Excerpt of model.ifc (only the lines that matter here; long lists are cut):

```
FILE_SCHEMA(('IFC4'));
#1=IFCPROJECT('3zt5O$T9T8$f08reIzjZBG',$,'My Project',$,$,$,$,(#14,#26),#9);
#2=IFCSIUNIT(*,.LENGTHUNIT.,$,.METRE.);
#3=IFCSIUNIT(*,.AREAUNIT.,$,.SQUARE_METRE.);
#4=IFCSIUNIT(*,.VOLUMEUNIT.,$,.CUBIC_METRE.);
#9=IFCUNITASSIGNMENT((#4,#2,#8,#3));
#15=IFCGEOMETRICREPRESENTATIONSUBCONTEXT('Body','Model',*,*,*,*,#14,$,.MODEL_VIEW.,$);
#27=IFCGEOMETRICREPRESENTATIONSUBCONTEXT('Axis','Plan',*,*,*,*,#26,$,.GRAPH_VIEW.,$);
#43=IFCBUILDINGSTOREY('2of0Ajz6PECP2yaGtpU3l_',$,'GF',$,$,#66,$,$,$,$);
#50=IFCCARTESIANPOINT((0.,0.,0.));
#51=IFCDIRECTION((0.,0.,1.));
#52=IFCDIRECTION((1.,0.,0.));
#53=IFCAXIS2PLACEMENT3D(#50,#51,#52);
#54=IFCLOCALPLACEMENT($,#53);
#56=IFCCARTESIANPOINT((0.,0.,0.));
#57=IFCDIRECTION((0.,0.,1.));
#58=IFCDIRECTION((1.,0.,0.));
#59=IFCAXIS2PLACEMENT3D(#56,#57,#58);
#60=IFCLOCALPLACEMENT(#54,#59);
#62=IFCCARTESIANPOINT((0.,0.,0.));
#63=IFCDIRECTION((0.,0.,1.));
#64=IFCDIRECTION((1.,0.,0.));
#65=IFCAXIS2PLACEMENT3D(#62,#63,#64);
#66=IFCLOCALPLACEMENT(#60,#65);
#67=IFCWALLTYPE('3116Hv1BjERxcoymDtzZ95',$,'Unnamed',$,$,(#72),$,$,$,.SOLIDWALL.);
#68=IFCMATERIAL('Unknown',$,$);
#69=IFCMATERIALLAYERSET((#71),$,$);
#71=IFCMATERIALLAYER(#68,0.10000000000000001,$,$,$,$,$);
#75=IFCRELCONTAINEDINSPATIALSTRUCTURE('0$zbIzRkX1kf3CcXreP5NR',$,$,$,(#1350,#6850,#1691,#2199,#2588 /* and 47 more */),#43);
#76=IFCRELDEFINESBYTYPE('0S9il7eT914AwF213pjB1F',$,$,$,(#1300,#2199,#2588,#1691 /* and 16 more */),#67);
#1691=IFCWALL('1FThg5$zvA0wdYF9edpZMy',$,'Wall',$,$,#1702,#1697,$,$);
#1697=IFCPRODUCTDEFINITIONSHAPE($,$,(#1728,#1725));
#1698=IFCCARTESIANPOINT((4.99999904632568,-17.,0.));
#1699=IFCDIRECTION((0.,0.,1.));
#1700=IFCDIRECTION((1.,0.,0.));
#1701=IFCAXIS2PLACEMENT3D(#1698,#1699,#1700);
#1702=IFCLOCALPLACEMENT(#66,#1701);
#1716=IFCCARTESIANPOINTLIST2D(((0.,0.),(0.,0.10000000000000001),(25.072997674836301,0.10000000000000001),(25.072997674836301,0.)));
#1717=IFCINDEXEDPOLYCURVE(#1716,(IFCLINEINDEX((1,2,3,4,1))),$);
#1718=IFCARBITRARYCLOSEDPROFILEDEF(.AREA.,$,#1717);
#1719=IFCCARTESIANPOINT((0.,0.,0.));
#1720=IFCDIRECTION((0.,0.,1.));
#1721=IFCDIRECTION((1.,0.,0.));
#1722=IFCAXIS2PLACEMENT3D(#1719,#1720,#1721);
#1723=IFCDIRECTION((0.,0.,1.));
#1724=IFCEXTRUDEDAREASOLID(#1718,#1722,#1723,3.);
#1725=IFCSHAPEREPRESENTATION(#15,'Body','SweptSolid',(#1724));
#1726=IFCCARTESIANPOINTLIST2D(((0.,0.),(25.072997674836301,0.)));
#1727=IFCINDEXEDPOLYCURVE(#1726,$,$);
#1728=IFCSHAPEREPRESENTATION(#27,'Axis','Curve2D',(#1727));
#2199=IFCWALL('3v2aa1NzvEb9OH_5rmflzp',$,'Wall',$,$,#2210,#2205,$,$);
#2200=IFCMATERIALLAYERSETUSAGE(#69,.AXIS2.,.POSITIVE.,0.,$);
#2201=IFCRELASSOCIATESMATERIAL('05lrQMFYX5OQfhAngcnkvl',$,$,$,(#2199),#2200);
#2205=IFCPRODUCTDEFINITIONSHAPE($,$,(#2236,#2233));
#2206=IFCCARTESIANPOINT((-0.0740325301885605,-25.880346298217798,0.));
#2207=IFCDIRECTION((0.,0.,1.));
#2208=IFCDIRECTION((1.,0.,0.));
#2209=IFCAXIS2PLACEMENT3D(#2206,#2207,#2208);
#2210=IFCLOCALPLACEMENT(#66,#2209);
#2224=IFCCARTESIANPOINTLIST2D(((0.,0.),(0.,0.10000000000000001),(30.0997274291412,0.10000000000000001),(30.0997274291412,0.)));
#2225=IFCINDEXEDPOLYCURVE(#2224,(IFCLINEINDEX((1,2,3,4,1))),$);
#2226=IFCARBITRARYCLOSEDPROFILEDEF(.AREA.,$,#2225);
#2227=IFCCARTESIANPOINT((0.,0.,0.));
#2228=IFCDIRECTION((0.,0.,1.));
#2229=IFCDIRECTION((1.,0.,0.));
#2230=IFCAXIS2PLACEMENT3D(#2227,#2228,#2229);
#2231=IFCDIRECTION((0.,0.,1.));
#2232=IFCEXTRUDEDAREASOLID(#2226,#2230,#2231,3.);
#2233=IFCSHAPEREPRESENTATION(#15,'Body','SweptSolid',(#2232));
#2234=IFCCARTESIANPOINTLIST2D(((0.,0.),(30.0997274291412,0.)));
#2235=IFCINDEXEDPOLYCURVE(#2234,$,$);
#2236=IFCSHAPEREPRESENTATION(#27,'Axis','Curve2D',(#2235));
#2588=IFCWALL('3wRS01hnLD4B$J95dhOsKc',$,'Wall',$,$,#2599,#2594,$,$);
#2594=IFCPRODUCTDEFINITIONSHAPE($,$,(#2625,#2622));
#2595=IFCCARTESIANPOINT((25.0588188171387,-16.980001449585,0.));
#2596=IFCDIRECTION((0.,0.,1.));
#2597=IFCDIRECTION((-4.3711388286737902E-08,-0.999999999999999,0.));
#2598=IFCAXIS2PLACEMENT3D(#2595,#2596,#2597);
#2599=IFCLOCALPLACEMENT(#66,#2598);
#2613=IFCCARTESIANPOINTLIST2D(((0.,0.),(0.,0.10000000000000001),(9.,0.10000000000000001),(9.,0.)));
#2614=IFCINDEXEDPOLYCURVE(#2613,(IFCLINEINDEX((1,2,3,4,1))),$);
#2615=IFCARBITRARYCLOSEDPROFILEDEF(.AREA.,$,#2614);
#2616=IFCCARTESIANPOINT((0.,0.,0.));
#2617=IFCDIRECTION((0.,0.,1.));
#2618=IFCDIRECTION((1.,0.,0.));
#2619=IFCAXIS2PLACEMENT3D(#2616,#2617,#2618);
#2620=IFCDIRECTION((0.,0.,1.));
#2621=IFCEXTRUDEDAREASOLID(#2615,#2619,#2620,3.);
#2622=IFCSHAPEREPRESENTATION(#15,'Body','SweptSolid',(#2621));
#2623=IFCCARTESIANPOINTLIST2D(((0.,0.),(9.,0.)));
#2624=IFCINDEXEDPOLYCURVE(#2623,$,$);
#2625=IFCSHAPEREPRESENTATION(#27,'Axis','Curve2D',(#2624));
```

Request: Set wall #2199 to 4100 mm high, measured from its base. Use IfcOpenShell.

```python
import ifcopenshell
import ifcopenshell.geom
import ifcopenshell.util.representation
import ifcopenshell.util.shape

model = ifcopenshell.open("model.ifc")
settings = ifcopenshell.geom.settings()


def volume(element):
    """Net volume in cubic metres, openings subtracted."""
    shape = ifcopenshell.geom.create_shape(settings, element)
    return ifcopenshell.util.shape.get_volume(shape.geometry)


wall = model.by_guid("3v2aa1NzvEb9OH_5rmflzp")
before = volume(wall)

body = ifcopenshell.util.representation.get_representation(wall, "Model", "Body")
solid = body.Items[0]
old_height = solid.Depth
solid.Depth = 4.1
after = volume(wall)

print(f"height {old_height:g} -> {solid.Depth:g}, volume {before:.3f} -> {after:.3f} m3")

model.write("model-out.ifc")
```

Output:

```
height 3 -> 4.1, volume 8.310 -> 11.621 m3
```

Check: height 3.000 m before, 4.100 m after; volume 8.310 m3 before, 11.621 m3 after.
